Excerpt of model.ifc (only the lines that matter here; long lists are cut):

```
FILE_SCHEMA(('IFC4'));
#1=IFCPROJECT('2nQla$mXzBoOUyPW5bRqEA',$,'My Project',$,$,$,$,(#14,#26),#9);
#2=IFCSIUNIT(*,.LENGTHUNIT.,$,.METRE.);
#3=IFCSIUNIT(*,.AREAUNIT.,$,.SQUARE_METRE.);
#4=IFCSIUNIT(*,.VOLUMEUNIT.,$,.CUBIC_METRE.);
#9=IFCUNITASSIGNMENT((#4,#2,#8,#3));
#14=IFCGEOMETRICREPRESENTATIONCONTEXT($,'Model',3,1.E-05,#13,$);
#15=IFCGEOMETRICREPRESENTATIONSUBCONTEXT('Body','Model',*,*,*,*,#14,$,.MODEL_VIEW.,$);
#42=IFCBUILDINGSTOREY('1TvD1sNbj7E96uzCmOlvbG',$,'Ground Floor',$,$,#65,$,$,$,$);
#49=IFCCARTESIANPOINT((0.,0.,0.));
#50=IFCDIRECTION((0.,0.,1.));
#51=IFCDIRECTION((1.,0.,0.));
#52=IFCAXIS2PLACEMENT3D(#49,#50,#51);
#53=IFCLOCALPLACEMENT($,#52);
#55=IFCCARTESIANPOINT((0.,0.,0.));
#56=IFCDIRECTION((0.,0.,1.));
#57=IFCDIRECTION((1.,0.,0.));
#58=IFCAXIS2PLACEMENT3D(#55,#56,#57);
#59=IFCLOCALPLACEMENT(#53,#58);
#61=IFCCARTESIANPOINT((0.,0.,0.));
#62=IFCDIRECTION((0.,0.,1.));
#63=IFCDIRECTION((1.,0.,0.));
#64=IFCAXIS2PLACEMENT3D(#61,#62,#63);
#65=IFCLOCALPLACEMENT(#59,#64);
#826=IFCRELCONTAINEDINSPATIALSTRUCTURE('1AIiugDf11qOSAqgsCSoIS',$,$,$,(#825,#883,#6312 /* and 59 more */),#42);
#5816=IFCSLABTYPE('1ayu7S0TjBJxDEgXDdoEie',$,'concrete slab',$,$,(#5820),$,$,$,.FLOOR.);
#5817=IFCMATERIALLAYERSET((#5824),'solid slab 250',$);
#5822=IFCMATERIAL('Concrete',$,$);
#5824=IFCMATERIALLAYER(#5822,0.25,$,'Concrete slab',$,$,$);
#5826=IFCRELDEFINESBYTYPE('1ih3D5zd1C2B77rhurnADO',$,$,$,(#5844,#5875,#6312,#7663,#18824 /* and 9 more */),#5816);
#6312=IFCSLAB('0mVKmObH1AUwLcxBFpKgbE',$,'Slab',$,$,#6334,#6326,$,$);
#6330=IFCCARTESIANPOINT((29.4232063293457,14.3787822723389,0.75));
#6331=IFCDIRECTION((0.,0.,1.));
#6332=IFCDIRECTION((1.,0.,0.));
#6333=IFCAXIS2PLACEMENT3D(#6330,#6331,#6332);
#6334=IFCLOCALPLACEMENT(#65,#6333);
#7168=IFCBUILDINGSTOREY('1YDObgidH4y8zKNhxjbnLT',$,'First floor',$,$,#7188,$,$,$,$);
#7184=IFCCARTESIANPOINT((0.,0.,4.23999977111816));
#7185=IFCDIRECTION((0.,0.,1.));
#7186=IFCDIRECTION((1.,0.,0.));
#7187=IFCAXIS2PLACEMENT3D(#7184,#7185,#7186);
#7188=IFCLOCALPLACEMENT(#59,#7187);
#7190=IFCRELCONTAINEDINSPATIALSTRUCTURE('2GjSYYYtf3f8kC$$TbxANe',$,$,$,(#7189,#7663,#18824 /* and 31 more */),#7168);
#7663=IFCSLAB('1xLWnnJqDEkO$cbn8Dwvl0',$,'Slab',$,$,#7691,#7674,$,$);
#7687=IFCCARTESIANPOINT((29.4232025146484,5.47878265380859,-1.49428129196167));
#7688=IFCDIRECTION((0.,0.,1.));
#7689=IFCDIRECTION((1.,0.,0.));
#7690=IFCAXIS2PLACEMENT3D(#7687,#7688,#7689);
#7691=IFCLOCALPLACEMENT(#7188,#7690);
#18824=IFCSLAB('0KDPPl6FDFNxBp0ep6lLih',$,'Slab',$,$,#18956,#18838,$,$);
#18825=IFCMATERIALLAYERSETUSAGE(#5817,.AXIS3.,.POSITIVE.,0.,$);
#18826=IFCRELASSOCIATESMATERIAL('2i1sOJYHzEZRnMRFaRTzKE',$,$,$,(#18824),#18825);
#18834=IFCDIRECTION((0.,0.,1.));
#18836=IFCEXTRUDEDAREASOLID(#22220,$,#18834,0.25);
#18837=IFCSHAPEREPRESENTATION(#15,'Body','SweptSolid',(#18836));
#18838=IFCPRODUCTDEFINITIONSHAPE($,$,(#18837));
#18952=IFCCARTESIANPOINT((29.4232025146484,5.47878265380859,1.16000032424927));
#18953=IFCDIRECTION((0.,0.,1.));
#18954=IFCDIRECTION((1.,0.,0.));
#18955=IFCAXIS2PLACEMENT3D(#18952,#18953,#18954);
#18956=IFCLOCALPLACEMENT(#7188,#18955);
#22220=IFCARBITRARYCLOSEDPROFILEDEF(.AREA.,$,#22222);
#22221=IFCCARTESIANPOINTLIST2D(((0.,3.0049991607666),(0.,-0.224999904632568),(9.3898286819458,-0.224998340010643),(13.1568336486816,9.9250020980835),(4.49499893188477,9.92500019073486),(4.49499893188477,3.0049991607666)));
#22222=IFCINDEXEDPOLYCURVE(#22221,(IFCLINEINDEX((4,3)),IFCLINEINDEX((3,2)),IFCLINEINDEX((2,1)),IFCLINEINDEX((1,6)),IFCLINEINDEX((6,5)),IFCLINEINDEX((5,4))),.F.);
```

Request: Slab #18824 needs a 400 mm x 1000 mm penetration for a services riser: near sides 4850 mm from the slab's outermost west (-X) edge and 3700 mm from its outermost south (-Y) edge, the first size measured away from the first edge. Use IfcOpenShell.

```python
import numpy as np
import ifcopenshell
import ifcopenshell.api.feature
import ifcopenshell.api.geometry
import ifcopenshell.api.root
import ifcopenshell.geom
import ifcopenshell.util.placement
import ifcopenshell.util.representation
import ifcopenshell.util.shape
import ifcopenshell.util.unit

model = ifcopenshell.open("model.ifc")
unit_scale = ifcopenshell.util.unit.calculate_unit_scale(model)
settings = ifcopenshell.geom.settings()


def volume(element):
    """Net volume in cubic metres, openings subtracted."""
    shape = ifcopenshell.geom.create_shape(settings, element)
    return ifcopenshell.util.shape.get_volume(shape.geometry)


slab = model.by_id(18824)
before = volume(slab)

# Extent in the slab's own axes, in metres. The edges named are its -X and -Y sides.
slab_shape = ifcopenshell.geom.create_shape(settings, slab)
vertices = ifcopenshell.util.shape.get_vertices(slab_shape.geometry)
x_min, y_min, bottom = vertices.min(axis=0)
top = vertices[:, 2].max()

opening = ifcopenshell.api.root.create_entity(model, ifc_class="IfcOpeningElement", name="Services riser opening", predefined_type="OPENING")
context = ifcopenshell.util.representation.get_context(model, "Model", "Body", "MODEL_VIEW")
width, depth = 0.4, 1
outline = [(0.0, 0.0), (width, 0.0), (width, depth), (0.0, depth), (0.0, 0.0)]
# Overshoot both faces by 50 mm so the cut is clean.
shape = ifcopenshell.api.geometry.add_slab_representation(
    model, context=context, depth=top - bottom + 0.1, polyline=outline
)
ifcopenshell.api.geometry.assign_representation(model, product=opening, representation=shape)

matrix = ifcopenshell.util.placement.get_local_placement(slab.ObjectPlacement)
matrix[:, 3] = matrix @ np.append(np.array([x_min + 4.85, y_min + 3.7, bottom - 0.05]) / unit_scale, 1.0)
ifcopenshell.api.geometry.edit_object_placement(model, product=opening, matrix=matrix, is_si=False)
ifcopenshell.api.feature.add_feature(model, feature=opening, element=slab)

after = volume(slab)

print(f"slab volume {before:.3f} -> {after:.3f} m3")

model.write("model_v2.ifc")
```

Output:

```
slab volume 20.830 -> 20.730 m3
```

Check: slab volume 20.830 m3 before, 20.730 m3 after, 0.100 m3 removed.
